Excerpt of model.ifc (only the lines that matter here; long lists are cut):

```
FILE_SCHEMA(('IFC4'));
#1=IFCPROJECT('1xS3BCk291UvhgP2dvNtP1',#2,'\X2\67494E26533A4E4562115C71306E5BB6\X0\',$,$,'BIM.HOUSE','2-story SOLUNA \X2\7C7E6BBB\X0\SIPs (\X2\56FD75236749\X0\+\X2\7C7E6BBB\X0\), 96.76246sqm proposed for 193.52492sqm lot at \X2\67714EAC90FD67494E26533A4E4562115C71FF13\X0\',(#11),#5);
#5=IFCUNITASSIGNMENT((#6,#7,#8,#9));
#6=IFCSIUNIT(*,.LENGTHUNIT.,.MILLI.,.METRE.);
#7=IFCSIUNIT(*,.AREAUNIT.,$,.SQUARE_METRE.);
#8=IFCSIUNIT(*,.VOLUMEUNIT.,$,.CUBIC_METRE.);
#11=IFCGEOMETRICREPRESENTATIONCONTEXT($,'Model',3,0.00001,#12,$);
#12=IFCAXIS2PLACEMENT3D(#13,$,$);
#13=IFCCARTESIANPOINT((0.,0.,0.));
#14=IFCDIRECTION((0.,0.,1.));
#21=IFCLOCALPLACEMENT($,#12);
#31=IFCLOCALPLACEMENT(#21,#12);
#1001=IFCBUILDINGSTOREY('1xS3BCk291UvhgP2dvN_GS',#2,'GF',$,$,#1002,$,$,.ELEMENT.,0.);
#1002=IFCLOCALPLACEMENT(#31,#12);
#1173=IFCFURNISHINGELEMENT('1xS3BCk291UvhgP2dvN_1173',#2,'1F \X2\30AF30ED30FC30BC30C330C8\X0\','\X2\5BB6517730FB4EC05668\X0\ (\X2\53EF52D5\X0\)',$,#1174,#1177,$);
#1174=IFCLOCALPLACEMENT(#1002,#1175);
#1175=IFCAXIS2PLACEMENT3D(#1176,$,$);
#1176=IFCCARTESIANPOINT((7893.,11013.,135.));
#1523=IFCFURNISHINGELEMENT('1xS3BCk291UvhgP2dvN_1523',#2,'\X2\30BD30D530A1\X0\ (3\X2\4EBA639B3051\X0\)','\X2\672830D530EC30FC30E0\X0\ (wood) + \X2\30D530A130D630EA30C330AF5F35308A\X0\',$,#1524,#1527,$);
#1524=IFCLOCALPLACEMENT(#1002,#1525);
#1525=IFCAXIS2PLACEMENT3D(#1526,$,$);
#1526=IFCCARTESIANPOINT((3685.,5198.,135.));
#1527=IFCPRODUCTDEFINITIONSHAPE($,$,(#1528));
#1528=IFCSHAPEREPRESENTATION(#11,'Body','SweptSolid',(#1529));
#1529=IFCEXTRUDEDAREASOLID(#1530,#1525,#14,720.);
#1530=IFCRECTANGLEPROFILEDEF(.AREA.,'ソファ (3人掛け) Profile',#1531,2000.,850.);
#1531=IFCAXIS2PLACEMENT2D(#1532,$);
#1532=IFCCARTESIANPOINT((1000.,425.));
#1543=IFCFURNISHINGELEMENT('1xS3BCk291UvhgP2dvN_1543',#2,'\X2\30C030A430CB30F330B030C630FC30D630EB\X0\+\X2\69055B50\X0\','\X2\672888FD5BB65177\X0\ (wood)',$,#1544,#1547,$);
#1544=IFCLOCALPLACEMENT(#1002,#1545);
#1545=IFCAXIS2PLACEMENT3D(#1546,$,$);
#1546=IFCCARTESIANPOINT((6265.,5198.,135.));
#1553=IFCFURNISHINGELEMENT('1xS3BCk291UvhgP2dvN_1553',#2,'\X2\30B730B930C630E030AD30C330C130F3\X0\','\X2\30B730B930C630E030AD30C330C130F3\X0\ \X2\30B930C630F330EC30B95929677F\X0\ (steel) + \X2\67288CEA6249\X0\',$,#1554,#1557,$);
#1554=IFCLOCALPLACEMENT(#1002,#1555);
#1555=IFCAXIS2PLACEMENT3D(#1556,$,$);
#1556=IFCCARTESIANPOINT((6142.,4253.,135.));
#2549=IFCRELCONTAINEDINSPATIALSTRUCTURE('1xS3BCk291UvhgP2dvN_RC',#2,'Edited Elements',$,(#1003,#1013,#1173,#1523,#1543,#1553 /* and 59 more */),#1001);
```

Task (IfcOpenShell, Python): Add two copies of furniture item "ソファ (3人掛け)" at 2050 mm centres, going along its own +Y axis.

```python
import ifcopenshell
import ifcopenshell.api.geometry
import ifcopenshell.api.root
import ifcopenshell.util.element
import ifcopenshell.util.placement
import ifcopenshell.util.unit

model = ifcopenshell.open("model.ifc")
unit_scale = ifcopenshell.util.unit.calculate_unit_scale(model)


def reuse_history(source, copy):
    """copy_class also copies each property set's owner history, people and application; keep the originals."""
    for rel in copy.IsDefinedBy:
        if rel.is_a("IfcRelDefinesByProperties") and (history := rel.RelatingPropertyDefinition.OwnerHistory):
            rel.RelatingPropertyDefinition.OwnerHistory = source.OwnerHistory
            ifcopenshell.util.element.remove_deep2(model, history)


source = model.by_guid("1xS3BCk291UvhgP2dvN_1523")
base = ifcopenshell.util.placement.get_local_placement(source.ObjectPlacement)
step = base[:3, 1] * 2.05 / unit_scale

for i in range(1, 3):
    copy = ifcopenshell.api.root.copy_class(model, product=source)
    copy.Representation = ifcopenshell.util.element.copy_deep(
        model, source.Representation, exclude=["IfcGeometricRepresentationContext", "IfcRepresentationMap"]
    )
    reuse_history(source, copy)
    matrix = base.copy()
    matrix[:3, 3] += i * step
    print("added at", matrix[:3, 3].round(3) + 0.0)
    ifcopenshell.api.geometry.edit_object_placement(model, product=copy, matrix=matrix, is_si=False)

model.write("model_edited.ifc")
```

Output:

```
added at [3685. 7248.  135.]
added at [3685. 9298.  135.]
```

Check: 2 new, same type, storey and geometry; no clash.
